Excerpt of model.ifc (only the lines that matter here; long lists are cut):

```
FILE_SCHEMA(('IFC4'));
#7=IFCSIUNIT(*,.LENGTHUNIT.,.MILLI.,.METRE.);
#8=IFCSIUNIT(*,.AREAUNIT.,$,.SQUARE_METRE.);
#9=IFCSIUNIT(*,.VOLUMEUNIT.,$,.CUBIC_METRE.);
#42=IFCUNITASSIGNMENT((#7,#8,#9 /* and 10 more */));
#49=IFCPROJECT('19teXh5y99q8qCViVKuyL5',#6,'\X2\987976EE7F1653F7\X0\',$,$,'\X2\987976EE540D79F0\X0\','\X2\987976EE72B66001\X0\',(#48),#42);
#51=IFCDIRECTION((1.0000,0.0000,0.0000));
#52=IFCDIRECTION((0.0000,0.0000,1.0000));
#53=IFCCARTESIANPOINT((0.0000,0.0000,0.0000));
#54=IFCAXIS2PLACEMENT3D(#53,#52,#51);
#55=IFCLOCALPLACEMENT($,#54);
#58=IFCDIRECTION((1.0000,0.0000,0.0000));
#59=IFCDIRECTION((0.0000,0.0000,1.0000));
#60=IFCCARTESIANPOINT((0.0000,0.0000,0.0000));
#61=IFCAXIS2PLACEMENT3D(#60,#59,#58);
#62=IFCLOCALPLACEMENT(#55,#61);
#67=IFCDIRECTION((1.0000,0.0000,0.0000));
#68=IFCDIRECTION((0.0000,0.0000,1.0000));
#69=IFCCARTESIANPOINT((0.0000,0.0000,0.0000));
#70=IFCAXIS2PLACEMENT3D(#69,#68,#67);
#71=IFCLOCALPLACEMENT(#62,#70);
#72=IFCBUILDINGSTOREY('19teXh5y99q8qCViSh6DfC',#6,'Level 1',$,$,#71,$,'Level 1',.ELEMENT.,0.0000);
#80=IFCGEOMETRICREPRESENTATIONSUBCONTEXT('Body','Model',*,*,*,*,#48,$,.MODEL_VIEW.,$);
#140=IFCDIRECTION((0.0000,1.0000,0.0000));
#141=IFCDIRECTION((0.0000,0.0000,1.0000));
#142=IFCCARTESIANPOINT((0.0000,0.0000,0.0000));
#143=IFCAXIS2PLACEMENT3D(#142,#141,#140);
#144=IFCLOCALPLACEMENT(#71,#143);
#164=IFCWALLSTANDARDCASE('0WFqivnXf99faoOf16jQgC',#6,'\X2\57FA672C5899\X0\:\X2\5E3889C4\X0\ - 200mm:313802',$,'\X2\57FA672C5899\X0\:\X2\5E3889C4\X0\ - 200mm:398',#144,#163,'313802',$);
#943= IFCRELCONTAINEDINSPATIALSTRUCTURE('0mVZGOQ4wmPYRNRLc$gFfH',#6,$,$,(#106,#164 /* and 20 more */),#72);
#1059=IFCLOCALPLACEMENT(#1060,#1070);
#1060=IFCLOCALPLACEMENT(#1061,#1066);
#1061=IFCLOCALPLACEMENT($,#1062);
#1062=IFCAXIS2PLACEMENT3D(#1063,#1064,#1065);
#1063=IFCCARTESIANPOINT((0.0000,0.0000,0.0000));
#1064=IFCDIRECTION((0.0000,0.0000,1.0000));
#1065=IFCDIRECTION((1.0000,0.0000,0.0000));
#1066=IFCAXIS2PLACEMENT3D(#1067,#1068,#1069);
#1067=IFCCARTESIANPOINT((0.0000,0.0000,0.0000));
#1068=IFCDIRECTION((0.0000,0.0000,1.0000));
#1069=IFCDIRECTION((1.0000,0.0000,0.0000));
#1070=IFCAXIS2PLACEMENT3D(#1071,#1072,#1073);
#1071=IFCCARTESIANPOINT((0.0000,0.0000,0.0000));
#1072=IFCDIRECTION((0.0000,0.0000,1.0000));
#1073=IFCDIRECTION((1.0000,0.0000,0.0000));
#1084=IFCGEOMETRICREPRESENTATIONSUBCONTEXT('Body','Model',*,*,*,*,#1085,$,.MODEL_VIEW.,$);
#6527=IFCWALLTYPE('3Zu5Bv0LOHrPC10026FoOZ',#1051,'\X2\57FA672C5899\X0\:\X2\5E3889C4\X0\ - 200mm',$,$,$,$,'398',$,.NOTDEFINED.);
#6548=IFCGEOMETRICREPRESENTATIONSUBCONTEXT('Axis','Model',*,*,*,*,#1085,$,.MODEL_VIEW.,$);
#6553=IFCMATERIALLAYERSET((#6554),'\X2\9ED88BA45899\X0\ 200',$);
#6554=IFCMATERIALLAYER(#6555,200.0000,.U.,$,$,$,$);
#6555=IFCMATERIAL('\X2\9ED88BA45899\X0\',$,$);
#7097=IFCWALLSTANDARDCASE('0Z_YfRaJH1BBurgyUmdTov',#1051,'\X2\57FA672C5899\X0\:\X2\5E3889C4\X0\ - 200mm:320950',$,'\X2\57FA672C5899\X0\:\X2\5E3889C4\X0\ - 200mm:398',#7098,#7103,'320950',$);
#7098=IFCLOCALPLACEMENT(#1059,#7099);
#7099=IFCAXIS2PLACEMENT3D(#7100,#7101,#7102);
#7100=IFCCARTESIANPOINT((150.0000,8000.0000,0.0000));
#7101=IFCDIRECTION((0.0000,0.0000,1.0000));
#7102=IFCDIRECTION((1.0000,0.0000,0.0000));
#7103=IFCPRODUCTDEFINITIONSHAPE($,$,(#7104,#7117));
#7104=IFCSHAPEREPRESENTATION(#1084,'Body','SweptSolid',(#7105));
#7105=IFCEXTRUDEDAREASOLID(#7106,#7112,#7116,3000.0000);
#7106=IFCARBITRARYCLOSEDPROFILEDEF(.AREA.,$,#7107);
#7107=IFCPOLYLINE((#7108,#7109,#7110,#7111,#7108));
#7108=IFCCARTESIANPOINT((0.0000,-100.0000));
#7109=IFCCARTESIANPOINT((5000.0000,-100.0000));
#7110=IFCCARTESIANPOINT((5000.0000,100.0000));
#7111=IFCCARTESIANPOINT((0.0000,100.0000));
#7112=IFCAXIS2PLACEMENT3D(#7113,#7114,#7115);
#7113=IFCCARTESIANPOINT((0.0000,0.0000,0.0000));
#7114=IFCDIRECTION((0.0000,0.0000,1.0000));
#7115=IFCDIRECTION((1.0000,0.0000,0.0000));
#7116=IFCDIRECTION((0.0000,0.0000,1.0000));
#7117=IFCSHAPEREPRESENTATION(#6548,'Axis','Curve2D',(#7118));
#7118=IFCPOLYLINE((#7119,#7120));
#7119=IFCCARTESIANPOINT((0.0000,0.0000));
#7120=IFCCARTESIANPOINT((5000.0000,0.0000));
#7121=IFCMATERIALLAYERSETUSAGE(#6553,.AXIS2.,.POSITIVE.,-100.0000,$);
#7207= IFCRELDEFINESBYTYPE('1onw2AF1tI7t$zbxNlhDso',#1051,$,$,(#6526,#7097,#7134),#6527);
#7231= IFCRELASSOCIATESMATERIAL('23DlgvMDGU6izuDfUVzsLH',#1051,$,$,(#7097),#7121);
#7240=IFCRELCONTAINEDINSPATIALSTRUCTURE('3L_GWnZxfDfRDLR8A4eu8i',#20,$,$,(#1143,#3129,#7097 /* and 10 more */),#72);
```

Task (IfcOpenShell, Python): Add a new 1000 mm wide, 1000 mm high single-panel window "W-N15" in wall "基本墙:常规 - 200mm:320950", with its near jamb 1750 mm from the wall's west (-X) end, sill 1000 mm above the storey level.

```python
import numpy as np
import ifcopenshell
import ifcopenshell.api.feature
import ifcopenshell.api.geometry
import ifcopenshell.api.root
import ifcopenshell.api.spatial
import ifcopenshell.geom
import ifcopenshell.util.element
import ifcopenshell.util.placement
import ifcopenshell.util.representation
import ifcopenshell.util.shape
import ifcopenshell.util.unit

model = ifcopenshell.open("model.ifc")
unit_scale = ifcopenshell.util.unit.calculate_unit_scale(model)
settings = ifcopenshell.geom.settings()


def volume(element):
    """Net volume in cubic metres, openings subtracted."""
    shape = ifcopenshell.geom.create_shape(settings, element)
    return ifcopenshell.util.shape.get_volume(shape.geometry)


wall = model.by_id(7097)
storey = ifcopenshell.util.element.get_container(wall, ifc_class="IfcBuildingStorey")
context = ifcopenshell.util.representation.get_context(model, "Model", "Body", "MODEL_VIEW")
before = volume(wall)

width, height, from_end, sill = 1, 1, 1.75, 1  # metres

# The wall runs along its own X axis, and the end named is its -X end.
wall_shape = ifcopenshell.geom.create_shape(settings, wall)
x, y, z = ifcopenshell.util.shape.get_vertices(wall_shape.geometry).T
start = x.min() + from_end
face, thickness = float(y.min()), float(y.max() - y.min())
wall_matrix = ifcopenshell.util.placement.get_local_placement(wall.ObjectPlacement)
level = ifcopenshell.util.placement.get_local_placement(storey.ObjectPlacement)[2, 3]


def in_wall(x, y):
    """Placement at x, y metres in the wall's axes, at sill height."""
    matrix = wall_matrix.copy()
    matrix[:, 3] = wall_matrix @ np.array([x / unit_scale, y / unit_scale, 0.0, 1.0])
    matrix[2, 3] = level + sill / unit_scale
    return matrix


# Opening: a box that overshoots both wall faces by 50 mm.
opening = ifcopenshell.api.root.create_entity(model, ifc_class="IfcOpeningElement", predefined_type="OPENING")
box = ifcopenshell.api.geometry.add_wall_representation(
    model, context=context, length=width, height=height, thickness=thickness + 0.1
)
ifcopenshell.api.geometry.assign_representation(model, product=opening, representation=box)
ifcopenshell.api.geometry.edit_object_placement(model, product=opening, matrix=in_wall(start, face - 0.05), is_si=False)
ifcopenshell.api.feature.add_feature(model, feature=opening, element=wall)

window = ifcopenshell.api.root.create_entity(model, ifc_class="IfcWindow", name="W-N15", predefined_type="WINDOW")
window.OverallWidth, window.OverallHeight = width / unit_scale, height / unit_scale
window.PartitioningType = "SINGLE_PANEL"
body = ifcopenshell.api.geometry.add_window_representation(
    model,
    context=context,
    overall_width=window.OverallWidth,
    overall_height=window.OverallHeight,
    partition_type="SINGLE_PANEL",
)
ifcopenshell.api.geometry.assign_representation(model, product=window, representation=body)
ifcopenshell.api.spatial.assign_container(model, products=[window], relating_structure=storey)
ifcopenshell.api.feature.add_filling(model, opening=opening, element=window)

# Centre the window in the wall's thickness.
ifcopenshell.api.geometry.edit_object_placement(model, product=window, matrix=in_wall(start, face), is_si=False)
window_shape = ifcopenshell.geom.create_shape(settings, window)
depth = ifcopenshell.util.shape.get_vertices(window_shape.geometry)[:, 1]
offset = face + thickness / 2 - (depth.min() + depth.max()) / 2
ifcopenshell.api.geometry.edit_object_placement(model, product=window, matrix=in_wall(start, offset), is_si=False)

after = volume(wall)

print(f"wall volume {before:.3f} -> {after:.3f} m3")

model.write("model_edited.ifc")
```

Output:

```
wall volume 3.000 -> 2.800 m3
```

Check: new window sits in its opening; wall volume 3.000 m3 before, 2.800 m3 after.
